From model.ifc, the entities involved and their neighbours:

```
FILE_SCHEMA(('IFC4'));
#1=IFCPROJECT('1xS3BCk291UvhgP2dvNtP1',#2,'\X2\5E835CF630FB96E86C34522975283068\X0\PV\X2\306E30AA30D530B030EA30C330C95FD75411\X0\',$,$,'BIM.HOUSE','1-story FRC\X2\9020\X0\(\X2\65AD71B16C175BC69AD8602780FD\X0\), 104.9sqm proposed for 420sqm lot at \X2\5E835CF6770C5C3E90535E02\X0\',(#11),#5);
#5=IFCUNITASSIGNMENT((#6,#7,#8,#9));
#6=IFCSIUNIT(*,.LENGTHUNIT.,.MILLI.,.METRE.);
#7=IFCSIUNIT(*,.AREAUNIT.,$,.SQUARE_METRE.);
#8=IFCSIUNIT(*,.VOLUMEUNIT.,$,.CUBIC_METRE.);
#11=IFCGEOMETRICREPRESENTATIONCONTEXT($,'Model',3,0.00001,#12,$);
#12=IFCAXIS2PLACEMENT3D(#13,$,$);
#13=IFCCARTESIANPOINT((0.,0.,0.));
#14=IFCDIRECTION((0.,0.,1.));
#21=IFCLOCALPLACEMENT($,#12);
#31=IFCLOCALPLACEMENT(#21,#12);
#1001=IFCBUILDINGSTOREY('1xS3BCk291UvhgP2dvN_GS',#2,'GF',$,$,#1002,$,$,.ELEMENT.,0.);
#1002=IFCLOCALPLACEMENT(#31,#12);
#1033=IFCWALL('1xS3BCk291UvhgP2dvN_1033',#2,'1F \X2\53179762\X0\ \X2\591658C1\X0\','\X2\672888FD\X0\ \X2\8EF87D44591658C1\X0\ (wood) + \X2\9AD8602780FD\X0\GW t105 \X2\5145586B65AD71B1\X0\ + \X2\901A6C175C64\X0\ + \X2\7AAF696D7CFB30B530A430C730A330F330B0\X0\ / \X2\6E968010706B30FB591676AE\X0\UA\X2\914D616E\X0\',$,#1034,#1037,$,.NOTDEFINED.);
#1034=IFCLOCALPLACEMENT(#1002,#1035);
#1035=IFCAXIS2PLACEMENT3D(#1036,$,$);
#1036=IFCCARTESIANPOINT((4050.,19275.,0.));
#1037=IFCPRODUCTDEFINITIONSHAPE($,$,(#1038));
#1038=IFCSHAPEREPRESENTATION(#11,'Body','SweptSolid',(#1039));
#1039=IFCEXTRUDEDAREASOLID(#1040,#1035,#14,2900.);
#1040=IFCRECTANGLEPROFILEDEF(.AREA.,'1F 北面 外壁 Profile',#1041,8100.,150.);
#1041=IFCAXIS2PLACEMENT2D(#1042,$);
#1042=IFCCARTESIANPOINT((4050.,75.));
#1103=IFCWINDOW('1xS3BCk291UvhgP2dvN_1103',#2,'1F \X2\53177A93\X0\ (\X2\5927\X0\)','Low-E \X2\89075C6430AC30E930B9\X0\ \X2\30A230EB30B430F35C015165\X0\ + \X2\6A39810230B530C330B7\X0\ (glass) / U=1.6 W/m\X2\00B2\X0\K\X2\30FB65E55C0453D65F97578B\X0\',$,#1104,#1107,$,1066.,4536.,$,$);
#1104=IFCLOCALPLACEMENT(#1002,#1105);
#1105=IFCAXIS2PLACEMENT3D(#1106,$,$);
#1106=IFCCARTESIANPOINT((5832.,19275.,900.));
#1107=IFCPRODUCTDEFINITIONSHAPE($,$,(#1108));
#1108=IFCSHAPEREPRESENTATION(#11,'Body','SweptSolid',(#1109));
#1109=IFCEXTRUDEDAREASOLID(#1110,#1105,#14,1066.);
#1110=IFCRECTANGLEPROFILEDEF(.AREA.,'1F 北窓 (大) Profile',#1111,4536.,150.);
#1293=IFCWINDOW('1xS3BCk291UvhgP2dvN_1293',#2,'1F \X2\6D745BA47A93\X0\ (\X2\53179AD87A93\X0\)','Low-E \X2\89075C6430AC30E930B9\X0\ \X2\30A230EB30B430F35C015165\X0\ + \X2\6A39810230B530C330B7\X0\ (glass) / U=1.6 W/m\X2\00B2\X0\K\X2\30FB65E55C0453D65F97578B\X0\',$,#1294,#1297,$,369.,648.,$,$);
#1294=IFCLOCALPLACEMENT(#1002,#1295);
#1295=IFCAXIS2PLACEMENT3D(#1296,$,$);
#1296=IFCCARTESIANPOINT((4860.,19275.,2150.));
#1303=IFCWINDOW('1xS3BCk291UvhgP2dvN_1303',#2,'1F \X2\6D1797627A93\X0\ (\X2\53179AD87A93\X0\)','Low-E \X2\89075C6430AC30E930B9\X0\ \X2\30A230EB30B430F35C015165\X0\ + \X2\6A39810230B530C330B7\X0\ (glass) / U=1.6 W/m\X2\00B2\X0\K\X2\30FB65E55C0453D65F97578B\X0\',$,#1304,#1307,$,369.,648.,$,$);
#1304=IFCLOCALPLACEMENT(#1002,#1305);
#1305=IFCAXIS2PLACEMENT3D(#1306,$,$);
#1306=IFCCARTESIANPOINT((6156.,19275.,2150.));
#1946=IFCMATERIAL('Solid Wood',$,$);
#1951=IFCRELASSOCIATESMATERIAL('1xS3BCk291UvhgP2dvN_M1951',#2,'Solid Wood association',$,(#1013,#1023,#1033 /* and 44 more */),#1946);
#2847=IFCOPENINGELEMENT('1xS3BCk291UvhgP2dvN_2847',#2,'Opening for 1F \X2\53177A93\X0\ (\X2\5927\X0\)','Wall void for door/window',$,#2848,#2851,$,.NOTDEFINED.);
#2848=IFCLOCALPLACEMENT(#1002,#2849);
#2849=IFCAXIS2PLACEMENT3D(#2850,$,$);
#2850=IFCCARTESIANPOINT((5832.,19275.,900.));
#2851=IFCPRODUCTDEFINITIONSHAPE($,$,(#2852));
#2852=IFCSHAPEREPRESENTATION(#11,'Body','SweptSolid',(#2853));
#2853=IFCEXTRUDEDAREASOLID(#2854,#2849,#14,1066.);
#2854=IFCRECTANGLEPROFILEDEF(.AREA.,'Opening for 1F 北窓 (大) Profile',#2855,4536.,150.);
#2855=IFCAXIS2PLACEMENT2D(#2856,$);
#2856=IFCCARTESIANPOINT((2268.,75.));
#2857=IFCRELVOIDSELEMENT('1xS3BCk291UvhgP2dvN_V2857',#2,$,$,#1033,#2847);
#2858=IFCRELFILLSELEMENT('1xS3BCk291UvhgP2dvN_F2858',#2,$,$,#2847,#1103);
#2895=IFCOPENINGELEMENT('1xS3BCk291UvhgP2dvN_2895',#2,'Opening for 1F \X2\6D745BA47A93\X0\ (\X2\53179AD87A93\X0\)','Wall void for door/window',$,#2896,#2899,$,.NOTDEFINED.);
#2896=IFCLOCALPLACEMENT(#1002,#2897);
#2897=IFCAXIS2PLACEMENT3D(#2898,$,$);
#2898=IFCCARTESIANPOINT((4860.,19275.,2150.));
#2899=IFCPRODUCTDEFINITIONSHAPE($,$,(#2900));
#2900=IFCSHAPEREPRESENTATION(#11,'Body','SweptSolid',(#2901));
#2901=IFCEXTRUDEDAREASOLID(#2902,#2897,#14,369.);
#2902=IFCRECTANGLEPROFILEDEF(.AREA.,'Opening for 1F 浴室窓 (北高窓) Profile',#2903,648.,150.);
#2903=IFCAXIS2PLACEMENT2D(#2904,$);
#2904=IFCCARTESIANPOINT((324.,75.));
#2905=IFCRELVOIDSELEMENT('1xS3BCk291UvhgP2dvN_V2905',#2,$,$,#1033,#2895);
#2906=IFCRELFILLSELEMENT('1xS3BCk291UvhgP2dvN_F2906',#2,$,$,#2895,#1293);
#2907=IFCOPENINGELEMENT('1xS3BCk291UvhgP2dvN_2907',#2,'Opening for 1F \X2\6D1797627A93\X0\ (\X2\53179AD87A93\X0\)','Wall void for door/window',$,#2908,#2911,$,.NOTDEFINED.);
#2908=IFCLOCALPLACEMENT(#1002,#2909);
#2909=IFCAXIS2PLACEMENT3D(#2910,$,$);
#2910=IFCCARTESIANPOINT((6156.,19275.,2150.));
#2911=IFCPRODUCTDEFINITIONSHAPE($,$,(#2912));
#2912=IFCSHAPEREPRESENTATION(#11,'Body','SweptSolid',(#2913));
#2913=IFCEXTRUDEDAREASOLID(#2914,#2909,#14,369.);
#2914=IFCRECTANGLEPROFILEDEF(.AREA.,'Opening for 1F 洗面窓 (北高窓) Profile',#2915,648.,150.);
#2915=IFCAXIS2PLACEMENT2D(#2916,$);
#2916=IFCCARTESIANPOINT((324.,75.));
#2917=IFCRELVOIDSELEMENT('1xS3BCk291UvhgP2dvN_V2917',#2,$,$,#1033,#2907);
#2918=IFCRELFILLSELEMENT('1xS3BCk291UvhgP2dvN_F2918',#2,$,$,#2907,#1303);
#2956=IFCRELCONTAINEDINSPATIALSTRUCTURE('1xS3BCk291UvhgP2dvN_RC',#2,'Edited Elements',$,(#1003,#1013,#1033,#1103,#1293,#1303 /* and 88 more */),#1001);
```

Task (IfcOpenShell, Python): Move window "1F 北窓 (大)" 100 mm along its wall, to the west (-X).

```python
import ifcopenshell
import ifcopenshell.api.geometry
import ifcopenshell.util.placement

model = ifcopenshell.open("model.ifc")

window = model.by_guid("1xS3BCk291UvhgP2dvN_1103")
opening = window.FillsVoids[0].RelatingOpeningElement
wall = opening.VoidsElements[0].RelatingBuildingElement

wall_matrix = ifcopenshell.util.placement.get_local_placement(wall.ObjectPlacement)
shift = wall_matrix[:3, 0] * -100.0
before = ifcopenshell.util.placement.get_local_placement(window.ObjectPlacement)[:3, 3].copy()

# The window is not placed relative to its opening, so move both.
for product in (opening, window):
    matrix = ifcopenshell.util.placement.get_local_placement(product.ObjectPlacement)
    matrix[:3, 3] += shift
    ifcopenshell.api.geometry.edit_object_placement(model, product=product, matrix=matrix, is_si=False)

after = ifcopenshell.util.placement.get_local_placement(window.ObjectPlacement)[:3, 3]
print("window moved by", (after - before).round(3) + 0.0)

model.write("model-out.ifc")
```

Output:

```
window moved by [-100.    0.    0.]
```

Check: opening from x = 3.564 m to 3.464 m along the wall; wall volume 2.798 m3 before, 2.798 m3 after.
